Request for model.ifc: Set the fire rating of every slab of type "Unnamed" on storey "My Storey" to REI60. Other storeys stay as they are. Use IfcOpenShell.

First a look at what the model holds.

```python
import ifcopenshell
import ifcopenshell.util.element

model = ifcopenshell.open("model.ifc")
print(model.schema)
storey = next(s for s in model.by_type("IfcBuildingStorey") if s.Name == "My Storey")
slabs = [e for e in ifcopenshell.util.element.get_decomposition(storey) if e.is_a("IfcSlab")]
seen = {}
for e in slabs:
    element_type = ifcopenshell.util.element.get_type(e)
    key = (element_type.Name if element_type != e and element_type else None, ifcopenshell.util.element.get_pset(e, "Pset_SlabCommon", "FireRating"))
    seen[key] = seen.get(key, 0) + 1
for (name, value), count in sorted(seen.items(), key=str):
    print(count, "x", name, "|", value)
```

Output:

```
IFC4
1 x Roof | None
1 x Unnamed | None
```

```python
import ifcopenshell
import ifcopenshell.api.pset
import ifcopenshell.util.element

model = ifcopenshell.open("model.ifc")

storey = next(s for s in model.by_type("IfcBuildingStorey") if s.Name == "My Storey")
slabs = [e for e in ifcopenshell.util.element.get_decomposition(storey) if e.is_a("IfcSlab")]

count = 0
for e in slabs:
    element_type = ifcopenshell.util.element.get_type(e)
    if element_type in (None, e) or element_type.Name != "Unnamed":
        continue
    # add_pset returns the element's existing set when there is one.
    pset = ifcopenshell.api.pset.add_pset(model, product=e, name="Pset_SlabCommon")
    ifcopenshell.api.pset.edit_pset(model, pset=pset, properties={"FireRating": "REI60"})
    count += 1

print(count, "slabs updated")

model.write("model_v2.ifc")
```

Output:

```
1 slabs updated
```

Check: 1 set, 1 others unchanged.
